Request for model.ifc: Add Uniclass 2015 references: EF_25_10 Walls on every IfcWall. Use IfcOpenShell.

First a look at what the model holds.

```python
import ifcopenshell

model = ifcopenshell.open("model.ifc")
print(model.schema)
print("classifications:", [c.Name for c in model.by_type("IfcClassification")])
for ifc_class in ("IfcDoor", "IfcRoof", "IfcStair", "IfcWall", "IfcWindow"):
    print(ifc_class, len(model.by_type(ifc_class)))
```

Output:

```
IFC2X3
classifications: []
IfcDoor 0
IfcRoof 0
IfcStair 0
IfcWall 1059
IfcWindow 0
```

```python
import ifcopenshell
import ifcopenshell.api.classification

model = ifcopenshell.open("model.ifc")

# IFC2X3 requires Source and Edition and has no link from the project to the system.
system = model.create_entity("IfcClassification", Source="NBS", Edition="2015", Name="Uniclass 2015")

codes = {
    "IfcWall": ("EF_25_10", "Walls"),
}
for ifc_class, (code, name) in codes.items():
    products = model.by_type(ifc_class)
    ifcopenshell.api.classification.add_reference(
        model, products=products, classification=system, identification=code, name=name
    )
    print(code, len(products))

model.write("model-out.ifc")
```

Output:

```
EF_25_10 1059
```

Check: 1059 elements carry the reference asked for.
